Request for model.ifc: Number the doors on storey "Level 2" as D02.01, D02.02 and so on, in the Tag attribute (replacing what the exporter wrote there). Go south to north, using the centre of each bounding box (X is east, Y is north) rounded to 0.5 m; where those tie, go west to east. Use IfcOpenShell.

First a look at what the model holds.

```python
import ifcopenshell
import ifcopenshell.util.element
import ifcopenshell.util.placement

model = ifcopenshell.open("model.ifc")
print(model.schema)
storey = next(s for s in model.by_type("IfcBuildingStorey") if s.Name == "Level 2")
doors = [e for e in ifcopenshell.util.element.get_decomposition(storey) if e.is_a("IfcDoor")]
for e in sorted(doors, key=lambda e: e.id()):
    origin = ifcopenshell.util.placement.get_local_placement(e.ObjectPlacement)[:3, 3]
    print(e.id(), e.Tag, e.Name, origin.round(2) + 0.0, sep=" | ")
```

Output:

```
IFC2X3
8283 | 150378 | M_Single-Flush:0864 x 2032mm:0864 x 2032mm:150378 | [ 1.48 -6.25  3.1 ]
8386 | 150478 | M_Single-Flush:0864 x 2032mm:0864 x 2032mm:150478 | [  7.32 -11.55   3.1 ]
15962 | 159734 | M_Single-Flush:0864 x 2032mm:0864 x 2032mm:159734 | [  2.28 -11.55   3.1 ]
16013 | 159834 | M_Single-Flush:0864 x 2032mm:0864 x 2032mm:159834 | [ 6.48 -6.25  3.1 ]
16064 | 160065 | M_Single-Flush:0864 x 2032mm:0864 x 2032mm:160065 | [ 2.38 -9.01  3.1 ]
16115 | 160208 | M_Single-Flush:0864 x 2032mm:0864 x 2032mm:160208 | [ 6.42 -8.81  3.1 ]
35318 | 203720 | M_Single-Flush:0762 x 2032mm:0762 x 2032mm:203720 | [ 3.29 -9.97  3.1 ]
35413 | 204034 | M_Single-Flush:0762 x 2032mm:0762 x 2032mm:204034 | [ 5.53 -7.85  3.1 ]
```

```python
import ifcopenshell
import ifcopenshell.geom
import ifcopenshell.util.element
import ifcopenshell.util.shape

model = ifcopenshell.open("model.ifc")
settings = ifcopenshell.geom.settings()
settings.set("use-world-coords", True)


def centre(element):
    shape = ifcopenshell.geom.create_shape(settings, element)
    return ifcopenshell.util.shape.get_bbox_centroid(shape.geometry)


storey = next(s for s in model.by_type("IfcBuildingStorey") if s.Name == "Level 2")
doors = [e for e in ifcopenshell.util.element.get_decomposition(storey) if e.is_a("IfcDoor")]

# Insertion points can sit at a corner or the storey origin, so sort by the geometry (in metres).
centres = {e: centre(e) for e in doors}
doors.sort(key=lambda e: (round(centres[e][1] / 0.5), centres[e][0]))

for i, e in enumerate(doors, start=1):
    number = f"D02.{i:02d}"
    e.Tag = number
    print(e.id(), number)

model.write("model_rev.ifc")
```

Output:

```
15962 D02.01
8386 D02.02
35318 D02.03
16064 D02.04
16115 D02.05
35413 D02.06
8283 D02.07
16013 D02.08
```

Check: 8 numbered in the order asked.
